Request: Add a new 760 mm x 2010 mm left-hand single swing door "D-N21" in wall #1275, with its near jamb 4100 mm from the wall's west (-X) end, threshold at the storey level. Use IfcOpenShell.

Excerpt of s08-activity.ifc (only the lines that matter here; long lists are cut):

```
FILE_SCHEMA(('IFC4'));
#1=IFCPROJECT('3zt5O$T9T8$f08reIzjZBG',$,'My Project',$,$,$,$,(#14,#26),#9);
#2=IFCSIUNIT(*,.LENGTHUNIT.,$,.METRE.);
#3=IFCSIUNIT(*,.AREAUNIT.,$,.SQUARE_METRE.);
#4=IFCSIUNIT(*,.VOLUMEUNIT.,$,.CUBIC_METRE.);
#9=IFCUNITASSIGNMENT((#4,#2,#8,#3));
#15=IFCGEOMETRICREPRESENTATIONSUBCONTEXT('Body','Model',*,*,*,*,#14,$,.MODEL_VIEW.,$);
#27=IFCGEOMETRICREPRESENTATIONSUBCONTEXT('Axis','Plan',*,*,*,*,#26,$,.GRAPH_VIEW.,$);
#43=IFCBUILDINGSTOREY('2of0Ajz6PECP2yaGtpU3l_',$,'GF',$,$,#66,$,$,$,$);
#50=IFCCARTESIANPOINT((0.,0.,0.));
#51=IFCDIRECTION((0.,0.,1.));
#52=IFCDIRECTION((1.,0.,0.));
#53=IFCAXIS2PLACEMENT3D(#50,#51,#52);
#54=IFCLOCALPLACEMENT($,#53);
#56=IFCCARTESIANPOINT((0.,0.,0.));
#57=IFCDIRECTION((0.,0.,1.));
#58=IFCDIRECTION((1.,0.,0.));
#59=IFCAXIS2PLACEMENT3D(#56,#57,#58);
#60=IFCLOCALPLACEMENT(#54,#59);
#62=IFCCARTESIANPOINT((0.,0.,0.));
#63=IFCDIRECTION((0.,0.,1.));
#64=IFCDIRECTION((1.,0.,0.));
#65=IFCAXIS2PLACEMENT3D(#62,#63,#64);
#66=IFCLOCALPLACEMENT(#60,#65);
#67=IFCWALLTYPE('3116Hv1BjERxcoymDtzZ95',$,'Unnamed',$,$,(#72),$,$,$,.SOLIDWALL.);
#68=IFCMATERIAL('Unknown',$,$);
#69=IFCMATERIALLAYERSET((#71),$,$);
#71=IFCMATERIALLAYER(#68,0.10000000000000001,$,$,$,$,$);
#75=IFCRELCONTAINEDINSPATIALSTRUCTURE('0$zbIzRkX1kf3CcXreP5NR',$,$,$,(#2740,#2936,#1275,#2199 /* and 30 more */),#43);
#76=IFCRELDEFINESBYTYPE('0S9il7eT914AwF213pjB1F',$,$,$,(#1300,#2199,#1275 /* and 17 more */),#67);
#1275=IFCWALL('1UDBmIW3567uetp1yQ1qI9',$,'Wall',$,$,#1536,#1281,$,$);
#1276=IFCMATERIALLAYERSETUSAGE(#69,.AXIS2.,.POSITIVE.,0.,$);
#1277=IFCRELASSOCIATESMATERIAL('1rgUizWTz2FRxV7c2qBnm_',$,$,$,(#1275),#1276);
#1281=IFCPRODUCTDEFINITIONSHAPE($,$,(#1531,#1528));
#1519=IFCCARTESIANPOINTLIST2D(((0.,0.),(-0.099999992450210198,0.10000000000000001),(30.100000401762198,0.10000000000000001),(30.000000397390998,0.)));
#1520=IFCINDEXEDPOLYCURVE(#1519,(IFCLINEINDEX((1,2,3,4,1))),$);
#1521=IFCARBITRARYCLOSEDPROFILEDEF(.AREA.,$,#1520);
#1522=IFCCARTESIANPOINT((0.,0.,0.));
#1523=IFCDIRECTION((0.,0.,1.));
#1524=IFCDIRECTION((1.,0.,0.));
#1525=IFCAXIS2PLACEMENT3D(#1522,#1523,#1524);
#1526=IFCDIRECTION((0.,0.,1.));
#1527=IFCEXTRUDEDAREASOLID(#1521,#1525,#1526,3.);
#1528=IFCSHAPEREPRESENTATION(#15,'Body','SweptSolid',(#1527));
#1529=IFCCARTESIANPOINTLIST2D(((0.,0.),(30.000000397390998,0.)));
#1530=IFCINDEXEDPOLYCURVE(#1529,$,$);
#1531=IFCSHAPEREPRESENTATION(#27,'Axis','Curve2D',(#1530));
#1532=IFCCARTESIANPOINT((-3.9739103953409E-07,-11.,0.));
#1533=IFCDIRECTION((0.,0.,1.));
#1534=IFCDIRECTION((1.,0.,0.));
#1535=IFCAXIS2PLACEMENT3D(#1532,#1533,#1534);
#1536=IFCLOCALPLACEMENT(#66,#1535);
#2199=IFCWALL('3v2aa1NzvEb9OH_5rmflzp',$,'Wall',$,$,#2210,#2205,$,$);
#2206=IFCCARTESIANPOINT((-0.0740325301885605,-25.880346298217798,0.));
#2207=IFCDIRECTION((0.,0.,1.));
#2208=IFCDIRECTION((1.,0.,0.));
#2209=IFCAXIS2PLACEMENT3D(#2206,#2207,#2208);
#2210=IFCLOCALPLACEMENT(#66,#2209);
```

```python
import numpy as np
import ifcopenshell
import ifcopenshell.api.feature
import ifcopenshell.api.geometry
import ifcopenshell.api.root
import ifcopenshell.api.spatial
import ifcopenshell.geom
import ifcopenshell.util.element
import ifcopenshell.util.placement
import ifcopenshell.util.representation
import ifcopenshell.util.shape
import ifcopenshell.util.unit

model = ifcopenshell.open("s08-activity.ifc")
unit_scale = ifcopenshell.util.unit.calculate_unit_scale(model)
settings = ifcopenshell.geom.settings()


def volume(element):
    """Net volume in cubic metres, openings subtracted."""
    shape = ifcopenshell.geom.create_shape(settings, element)
    return ifcopenshell.util.shape.get_volume(shape.geometry)


wall = model.by_id(1275)
storey = ifcopenshell.util.element.get_container(wall, ifc_class="IfcBuildingStorey")
context = ifcopenshell.util.representation.get_context(model, "Model", "Body", "MODEL_VIEW")
before = volume(wall)

width, height, from_end, sill = 0.76, 2.01, 4.1, 0.0  # metres

# The wall runs along its own X axis, and the end named is its -X end.
wall_shape = ifcopenshell.geom.create_shape(settings, wall)
x, y, z = ifcopenshell.util.shape.get_vertices(wall_shape.geometry).T
start = x.min() + from_end
face, thickness = float(y.min()), float(y.max() - y.min())
wall_matrix = ifcopenshell.util.placement.get_local_placement(wall.ObjectPlacement)
level = ifcopenshell.util.placement.get_local_placement(storey.ObjectPlacement)[2, 3]


def in_wall(x, y):
    """Placement at x, y metres in the wall's axes, at sill height."""
    matrix = wall_matrix.copy()
    matrix[:, 3] = wall_matrix @ np.array([x / unit_scale, y / unit_scale, 0.0, 1.0])
    matrix[2, 3] = level + sill / unit_scale
    return matrix


# Opening: a box that overshoots both wall faces by 50 mm.
opening = ifcopenshell.api.root.create_entity(model, ifc_class="IfcOpeningElement", predefined_type="OPENING")
box = ifcopenshell.api.geometry.add_wall_representation(
    model, context=context, length=width, height=height, thickness=thickness + 0.1
)
ifcopenshell.api.geometry.assign_representation(model, product=opening, representation=box)
ifcopenshell.api.geometry.edit_object_placement(model, product=opening, matrix=in_wall(start, face - 0.05), is_si=False)
ifcopenshell.api.feature.add_feature(model, feature=opening, element=wall)

door = ifcopenshell.api.root.create_entity(model, ifc_class="IfcDoor", name="D-N21", predefined_type="DOOR")
door.OverallWidth, door.OverallHeight = width / unit_scale, height / unit_scale
door.OperationType = "SINGLE_SWING_LEFT"
body = ifcopenshell.api.geometry.add_door_representation(
    model,
    context=context,
    overall_width=door.OverallWidth,
    overall_height=door.OverallHeight,
    operation_type="SINGLE_SWING_LEFT",
    lining_properties={"LiningDepth": thickness / unit_scale, "ThresholdDepth": thickness / unit_scale},
)
ifcopenshell.api.geometry.assign_representation(model, product=door, representation=body)
ifcopenshell.api.spatial.assign_container(model, products=[door], relating_structure=storey)
ifcopenshell.api.feature.add_filling(model, opening=opening, element=door)

# The lining spans the wall, so the door starts at the wall face.
ifcopenshell.api.geometry.edit_object_placement(model, product=door, matrix=in_wall(start, face), is_si=False)

after = volume(wall)

print(f"wall volume {before:.3f} -> {after:.3f} m3")

model.write("s08-activity_v2.ifc")
```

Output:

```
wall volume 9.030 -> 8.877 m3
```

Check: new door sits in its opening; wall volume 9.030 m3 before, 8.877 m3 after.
